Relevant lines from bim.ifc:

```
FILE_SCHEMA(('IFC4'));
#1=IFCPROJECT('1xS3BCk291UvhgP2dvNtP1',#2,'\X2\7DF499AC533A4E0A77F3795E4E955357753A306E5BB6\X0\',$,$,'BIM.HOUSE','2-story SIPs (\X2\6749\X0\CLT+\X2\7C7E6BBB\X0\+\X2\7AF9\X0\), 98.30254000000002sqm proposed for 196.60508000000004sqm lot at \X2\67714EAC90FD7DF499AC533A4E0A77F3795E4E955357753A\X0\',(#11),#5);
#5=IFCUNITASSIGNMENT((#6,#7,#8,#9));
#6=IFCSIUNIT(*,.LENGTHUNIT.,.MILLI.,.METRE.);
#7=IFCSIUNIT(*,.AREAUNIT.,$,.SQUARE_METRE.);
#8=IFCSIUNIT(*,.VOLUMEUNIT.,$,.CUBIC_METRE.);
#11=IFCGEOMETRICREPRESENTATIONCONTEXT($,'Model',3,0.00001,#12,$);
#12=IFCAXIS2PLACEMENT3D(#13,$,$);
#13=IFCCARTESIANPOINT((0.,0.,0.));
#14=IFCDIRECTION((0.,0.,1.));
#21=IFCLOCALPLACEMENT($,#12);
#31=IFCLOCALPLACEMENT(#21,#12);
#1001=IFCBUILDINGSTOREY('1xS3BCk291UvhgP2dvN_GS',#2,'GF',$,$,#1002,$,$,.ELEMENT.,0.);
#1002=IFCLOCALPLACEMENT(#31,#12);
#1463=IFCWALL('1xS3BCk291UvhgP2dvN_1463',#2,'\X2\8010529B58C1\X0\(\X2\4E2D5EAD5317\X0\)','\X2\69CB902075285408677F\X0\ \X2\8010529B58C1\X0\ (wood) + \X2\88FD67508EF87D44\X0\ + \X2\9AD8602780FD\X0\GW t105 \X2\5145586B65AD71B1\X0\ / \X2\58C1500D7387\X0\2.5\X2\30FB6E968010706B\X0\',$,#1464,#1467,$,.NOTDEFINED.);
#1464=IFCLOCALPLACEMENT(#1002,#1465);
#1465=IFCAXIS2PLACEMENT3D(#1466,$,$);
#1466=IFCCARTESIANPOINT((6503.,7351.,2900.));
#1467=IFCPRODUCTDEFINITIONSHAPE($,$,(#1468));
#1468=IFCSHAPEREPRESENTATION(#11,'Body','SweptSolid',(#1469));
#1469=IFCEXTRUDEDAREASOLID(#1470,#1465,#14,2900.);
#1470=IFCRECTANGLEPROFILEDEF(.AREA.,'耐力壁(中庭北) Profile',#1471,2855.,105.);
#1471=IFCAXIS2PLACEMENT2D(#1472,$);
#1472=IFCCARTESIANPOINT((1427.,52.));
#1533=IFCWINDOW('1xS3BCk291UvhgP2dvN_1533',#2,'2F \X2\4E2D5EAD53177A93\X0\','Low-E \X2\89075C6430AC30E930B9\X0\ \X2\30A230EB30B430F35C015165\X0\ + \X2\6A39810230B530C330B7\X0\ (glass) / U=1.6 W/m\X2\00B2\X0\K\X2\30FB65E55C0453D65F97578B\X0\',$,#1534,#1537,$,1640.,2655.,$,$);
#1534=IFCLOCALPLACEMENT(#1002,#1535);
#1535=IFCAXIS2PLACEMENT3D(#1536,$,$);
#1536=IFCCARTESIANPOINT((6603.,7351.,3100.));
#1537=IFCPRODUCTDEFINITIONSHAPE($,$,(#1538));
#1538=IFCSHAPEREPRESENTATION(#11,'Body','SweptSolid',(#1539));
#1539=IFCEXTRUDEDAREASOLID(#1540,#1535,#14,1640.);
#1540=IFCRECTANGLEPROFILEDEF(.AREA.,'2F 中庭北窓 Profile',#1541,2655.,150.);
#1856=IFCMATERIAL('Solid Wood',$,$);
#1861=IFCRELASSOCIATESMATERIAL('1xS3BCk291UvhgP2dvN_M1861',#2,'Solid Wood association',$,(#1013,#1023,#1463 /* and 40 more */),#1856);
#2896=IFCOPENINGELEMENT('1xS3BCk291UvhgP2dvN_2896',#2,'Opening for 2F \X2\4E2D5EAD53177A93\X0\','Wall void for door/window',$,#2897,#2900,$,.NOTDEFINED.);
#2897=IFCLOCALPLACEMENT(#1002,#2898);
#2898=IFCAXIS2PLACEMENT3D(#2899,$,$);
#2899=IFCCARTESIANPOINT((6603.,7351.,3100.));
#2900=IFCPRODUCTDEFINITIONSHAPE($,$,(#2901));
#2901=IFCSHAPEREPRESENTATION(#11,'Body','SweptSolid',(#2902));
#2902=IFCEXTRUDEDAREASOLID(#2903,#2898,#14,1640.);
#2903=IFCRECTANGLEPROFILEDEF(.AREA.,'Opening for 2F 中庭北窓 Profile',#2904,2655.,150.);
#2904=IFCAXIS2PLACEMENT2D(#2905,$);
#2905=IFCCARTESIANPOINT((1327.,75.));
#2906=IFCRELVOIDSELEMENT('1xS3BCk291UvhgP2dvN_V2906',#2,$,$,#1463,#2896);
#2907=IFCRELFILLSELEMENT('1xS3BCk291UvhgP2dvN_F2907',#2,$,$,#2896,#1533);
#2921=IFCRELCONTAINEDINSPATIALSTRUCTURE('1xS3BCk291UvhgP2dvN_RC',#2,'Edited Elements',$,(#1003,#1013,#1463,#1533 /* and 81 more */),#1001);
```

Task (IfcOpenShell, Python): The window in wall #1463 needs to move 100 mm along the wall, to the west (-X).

```python
import ifcopenshell
import ifcopenshell.api.geometry
import ifcopenshell.util.placement
import ifcopenshell.util.unit

model = ifcopenshell.open("bim.ifc")
unit_scale = ifcopenshell.util.unit.calculate_unit_scale(model)

window = model.by_guid("1xS3BCk291UvhgP2dvN_1533")
opening = window.FillsVoids[0].RelatingOpeningElement
wall = opening.VoidsElements[0].RelatingBuildingElement

wall_matrix = ifcopenshell.util.placement.get_local_placement(wall.ObjectPlacement)
shift = wall_matrix[:3, 0] * -0.1 / unit_scale
before = ifcopenshell.util.placement.get_local_placement(window.ObjectPlacement)[:3, 3].copy()

# The window is not placed relative to its opening, so move both.
for product in (opening, window):
    matrix = ifcopenshell.util.placement.get_local_placement(product.ObjectPlacement)
    matrix[:3, 3] += shift
    ifcopenshell.api.geometry.edit_object_placement(model, product=product, matrix=matrix, is_si=False)

after = ifcopenshell.util.placement.get_local_placement(window.ObjectPlacement)[:3, 3]
print("window moved by", (after - before).round(3) + 0.0)

model.write("bim_edited.ifc")
```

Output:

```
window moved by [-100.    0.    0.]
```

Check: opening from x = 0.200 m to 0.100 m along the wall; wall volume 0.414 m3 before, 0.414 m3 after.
